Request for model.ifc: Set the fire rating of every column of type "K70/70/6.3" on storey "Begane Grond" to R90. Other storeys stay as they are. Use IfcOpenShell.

First a look at what the model holds.

```python
import ifcopenshell
import ifcopenshell.util.element

model = ifcopenshell.open("model.ifc")
print(model.schema)
storey = next(s for s in model.by_type("IfcBuildingStorey") if s.Name == "Begane Grond")
columns = [e for e in ifcopenshell.util.element.get_decomposition(storey) if e.is_a("IfcColumn")]
seen = {}
for e in columns:
    element_type = ifcopenshell.util.element.get_type(e)
    key = (element_type.Name if element_type != e and element_type else None, ifcopenshell.util.element.get_pset(e, "Pset_ColumnCommon", "FireRating"))
    seen[key] = seen.get(key, 0) + 1
for (name, value), count in sorted(seen.items(), key=str):
    print(count, "x", name, "|", value)
```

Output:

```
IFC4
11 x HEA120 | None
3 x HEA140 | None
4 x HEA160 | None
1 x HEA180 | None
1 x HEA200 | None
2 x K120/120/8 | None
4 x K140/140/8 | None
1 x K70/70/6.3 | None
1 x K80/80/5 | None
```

```python
import ifcopenshell
import ifcopenshell.api.pset
import ifcopenshell.util.element

model = ifcopenshell.open("model.ifc")

storey = next(s for s in model.by_type("IfcBuildingStorey") if s.Name == "Begane Grond")
columns = [e for e in ifcopenshell.util.element.get_decomposition(storey) if e.is_a("IfcColumn")]

count = 0
for e in columns:
    element_type = ifcopenshell.util.element.get_type(e)
    if element_type in (None, e) or element_type.Name != "K70/70/6.3":
        continue
    # add_pset returns the element's existing set when there is one.
    pset = ifcopenshell.api.pset.add_pset(model, product=e, name="Pset_ColumnCommon")
    ifcopenshell.api.pset.edit_pset(model, pset=pset, properties={"FireRating": "R90"})
    count += 1

print(count, "columns updated")

model.write("model_updated.ifc")
```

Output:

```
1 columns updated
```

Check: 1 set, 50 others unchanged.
